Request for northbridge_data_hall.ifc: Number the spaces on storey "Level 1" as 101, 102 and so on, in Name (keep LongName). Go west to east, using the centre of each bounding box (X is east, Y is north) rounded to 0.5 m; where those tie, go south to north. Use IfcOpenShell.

First a look at what the model holds.

```python
import ifcopenshell
import ifcopenshell.util.element
import ifcopenshell.util.placement

model = ifcopenshell.open("northbridge_data_hall.ifc")
print(model.schema)
storey = next(s for s in model.by_type("IfcBuildingStorey") if s.Name == "Level 1")
spaces = [e for e in ifcopenshell.util.element.get_decomposition(storey) if e.is_a("IfcSpace")]
for e in sorted(spaces, key=lambda e: e.id()):
    origin = ifcopenshell.util.placement.get_local_placement(e.ObjectPlacement)[:3, 3]
    print(e.id(), e.Name, e.LongName, origin.round(2) + 0.0, sep=" | ")
```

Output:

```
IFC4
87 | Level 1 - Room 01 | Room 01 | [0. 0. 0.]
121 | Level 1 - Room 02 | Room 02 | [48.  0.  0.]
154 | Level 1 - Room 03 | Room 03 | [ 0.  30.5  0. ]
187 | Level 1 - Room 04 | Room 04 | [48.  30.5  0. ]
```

```python
import ifcopenshell
import ifcopenshell.geom
import ifcopenshell.util.element
import ifcopenshell.util.shape

model = ifcopenshell.open("northbridge_data_hall.ifc")
settings = ifcopenshell.geom.settings()
settings.set("use-world-coords", True)


def centre(element):
    shape = ifcopenshell.geom.create_shape(settings, element)
    return ifcopenshell.util.shape.get_bbox_centroid(shape.geometry)


storey = next(s for s in model.by_type("IfcBuildingStorey") if s.Name == "Level 1")
spaces = [e for e in ifcopenshell.util.element.get_decomposition(storey) if e.is_a("IfcSpace")]

# Insertion points can sit at a corner or the storey origin, so sort by the geometry (in metres).
centres = {e: centre(e) for e in spaces}
spaces.sort(key=lambda e: (round(centres[e][0] / 0.5), centres[e][1]))

for i, e in enumerate(spaces, start=1):
    number = f"1{i:02d}"
    e.Name = number
    print(e.id(), number)

model.write("northbridge_data_hall_edited.ifc")
```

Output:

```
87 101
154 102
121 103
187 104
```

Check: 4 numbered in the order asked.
